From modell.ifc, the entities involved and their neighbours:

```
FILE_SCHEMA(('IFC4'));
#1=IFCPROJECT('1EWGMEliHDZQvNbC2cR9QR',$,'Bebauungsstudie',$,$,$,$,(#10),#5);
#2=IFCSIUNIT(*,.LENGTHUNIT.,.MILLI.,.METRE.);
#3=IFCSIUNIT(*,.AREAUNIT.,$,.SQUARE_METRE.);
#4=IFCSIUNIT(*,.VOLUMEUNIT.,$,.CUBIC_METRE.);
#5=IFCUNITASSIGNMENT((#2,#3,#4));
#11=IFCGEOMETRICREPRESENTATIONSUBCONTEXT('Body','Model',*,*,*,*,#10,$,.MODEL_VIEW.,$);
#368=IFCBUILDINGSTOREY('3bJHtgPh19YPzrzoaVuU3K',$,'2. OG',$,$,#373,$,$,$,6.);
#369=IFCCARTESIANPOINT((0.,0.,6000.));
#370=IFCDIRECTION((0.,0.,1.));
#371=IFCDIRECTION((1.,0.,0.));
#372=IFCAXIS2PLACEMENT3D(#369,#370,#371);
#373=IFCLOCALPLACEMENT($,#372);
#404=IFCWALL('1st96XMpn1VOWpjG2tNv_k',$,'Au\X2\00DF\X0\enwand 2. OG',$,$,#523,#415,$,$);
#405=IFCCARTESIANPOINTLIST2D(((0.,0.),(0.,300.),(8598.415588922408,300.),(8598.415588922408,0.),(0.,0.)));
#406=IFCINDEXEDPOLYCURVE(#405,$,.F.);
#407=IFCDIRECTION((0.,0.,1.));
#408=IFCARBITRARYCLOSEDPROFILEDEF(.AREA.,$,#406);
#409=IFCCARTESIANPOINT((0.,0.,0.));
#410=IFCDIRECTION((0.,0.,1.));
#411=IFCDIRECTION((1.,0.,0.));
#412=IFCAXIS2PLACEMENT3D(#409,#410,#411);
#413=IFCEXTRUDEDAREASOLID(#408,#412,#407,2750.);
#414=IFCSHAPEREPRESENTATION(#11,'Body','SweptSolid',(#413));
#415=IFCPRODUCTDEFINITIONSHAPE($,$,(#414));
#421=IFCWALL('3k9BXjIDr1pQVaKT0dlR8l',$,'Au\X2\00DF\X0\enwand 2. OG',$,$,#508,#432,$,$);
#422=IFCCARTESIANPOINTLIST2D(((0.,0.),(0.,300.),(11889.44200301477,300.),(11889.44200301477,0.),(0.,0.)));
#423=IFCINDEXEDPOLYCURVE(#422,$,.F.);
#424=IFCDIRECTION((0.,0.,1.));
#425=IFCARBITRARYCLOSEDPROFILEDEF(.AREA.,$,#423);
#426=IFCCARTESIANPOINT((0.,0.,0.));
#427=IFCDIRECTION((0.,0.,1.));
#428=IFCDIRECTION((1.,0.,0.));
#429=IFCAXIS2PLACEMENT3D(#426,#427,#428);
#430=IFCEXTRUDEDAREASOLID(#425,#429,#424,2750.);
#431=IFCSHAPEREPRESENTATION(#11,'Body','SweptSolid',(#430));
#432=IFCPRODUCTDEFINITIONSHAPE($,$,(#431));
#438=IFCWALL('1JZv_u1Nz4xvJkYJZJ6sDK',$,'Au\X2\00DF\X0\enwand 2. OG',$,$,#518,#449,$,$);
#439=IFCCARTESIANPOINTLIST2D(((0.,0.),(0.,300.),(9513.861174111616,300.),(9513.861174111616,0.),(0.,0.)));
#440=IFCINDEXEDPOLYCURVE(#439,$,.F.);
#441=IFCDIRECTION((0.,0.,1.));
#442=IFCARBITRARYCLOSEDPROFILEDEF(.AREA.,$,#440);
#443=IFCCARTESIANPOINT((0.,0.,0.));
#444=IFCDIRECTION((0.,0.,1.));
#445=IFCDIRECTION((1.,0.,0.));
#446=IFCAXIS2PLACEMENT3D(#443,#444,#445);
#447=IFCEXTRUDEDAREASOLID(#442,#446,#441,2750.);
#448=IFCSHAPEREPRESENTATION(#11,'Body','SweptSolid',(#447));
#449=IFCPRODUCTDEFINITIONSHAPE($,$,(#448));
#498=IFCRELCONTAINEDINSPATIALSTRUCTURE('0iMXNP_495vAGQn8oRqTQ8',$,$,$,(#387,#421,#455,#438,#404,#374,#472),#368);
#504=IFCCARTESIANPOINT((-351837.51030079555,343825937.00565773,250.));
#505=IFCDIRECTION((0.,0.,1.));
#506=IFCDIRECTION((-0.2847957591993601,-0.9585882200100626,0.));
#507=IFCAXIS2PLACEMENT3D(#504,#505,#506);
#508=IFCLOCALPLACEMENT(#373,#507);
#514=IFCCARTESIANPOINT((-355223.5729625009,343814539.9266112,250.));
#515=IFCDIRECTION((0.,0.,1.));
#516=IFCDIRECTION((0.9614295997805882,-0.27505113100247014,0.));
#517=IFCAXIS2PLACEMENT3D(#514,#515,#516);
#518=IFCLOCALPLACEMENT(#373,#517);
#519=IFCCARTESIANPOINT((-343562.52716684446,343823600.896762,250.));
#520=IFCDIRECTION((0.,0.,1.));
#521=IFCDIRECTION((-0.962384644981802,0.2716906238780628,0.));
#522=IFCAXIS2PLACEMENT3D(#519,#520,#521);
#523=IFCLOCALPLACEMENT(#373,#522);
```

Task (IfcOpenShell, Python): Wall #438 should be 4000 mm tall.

```python
import ifcopenshell
import ifcopenshell.geom
import ifcopenshell.util.representation
import ifcopenshell.util.shape
import ifcopenshell.util.unit

model = ifcopenshell.open("modell.ifc")
unit_scale = ifcopenshell.util.unit.calculate_unit_scale(model)
settings = ifcopenshell.geom.settings()


def volume(element):
    """Net volume in cubic metres, openings subtracted."""
    shape = ifcopenshell.geom.create_shape(settings, element)
    return ifcopenshell.util.shape.get_volume(shape.geometry)


wall = model.by_id(438)
before = volume(wall)

body = ifcopenshell.util.representation.get_representation(wall, "Model", "Body")
solid = body.Items[0]
old_height = solid.Depth
solid.Depth = 4 / unit_scale
after = volume(wall)

print(f"height {old_height:g} -> {solid.Depth:g}, volume {before:.3f} -> {after:.3f} m3")

model.write("modell_edited.ifc")
```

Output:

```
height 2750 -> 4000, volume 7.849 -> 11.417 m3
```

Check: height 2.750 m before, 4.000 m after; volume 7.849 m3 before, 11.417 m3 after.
